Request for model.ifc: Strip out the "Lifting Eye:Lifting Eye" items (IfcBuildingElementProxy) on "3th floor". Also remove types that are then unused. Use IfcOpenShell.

First a look at what the model holds.

```python
import ifcopenshell
import ifcopenshell.util.element

model = ifcopenshell.open("model.ifc")
print(model.schema)
storey = next(s for s in model.by_type("IfcBuildingStorey") if s.Name == "3th floor")
proxies = [e for e in ifcopenshell.util.element.get_decomposition(storey) if e.is_a("IfcBuildingElementProxy")]
seen = {}
for e in proxies:
    element_type = ifcopenshell.util.element.get_type(e)
    name = element_type.Name if element_type not in (None, e) else None
    seen[name] = seen.get(name, 0) + 1
for name, count in sorted(seen.items(), key=str):
    print(count, "x", name)
```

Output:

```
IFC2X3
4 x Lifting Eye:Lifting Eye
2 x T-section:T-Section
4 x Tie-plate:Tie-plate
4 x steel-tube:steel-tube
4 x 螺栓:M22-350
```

```python
import ifcopenshell
import ifcopenshell.api.root
import ifcopenshell.util.element

model = ifcopenshell.open("model.ifc")

storey = next(s for s in model.by_type("IfcBuildingStorey") if s.Name == "3th floor")
proxies = [e for e in ifcopenshell.util.element.get_decomposition(storey) if e.is_a("IfcBuildingElementProxy")]
targets = [e for e in proxies if (t := ifcopenshell.util.element.get_type(e)) not in (None, e) and t.Name == "Lifting Eye:Lifting Eye"]
types = {ifcopenshell.util.element.get_type(e) for e in targets} - {None, *targets}

for e in targets:
    ifcopenshell.api.root.remove_product(model, product=e)
print(len(targets), "removed")

unused = [t for t in types if not ifcopenshell.util.element.get_types(t)]
for t in unused:
    ifcopenshell.api.root.remove_product(model, product=t)
print(len(unused), "unused types removed")

model.write("model_updated.ifc")
```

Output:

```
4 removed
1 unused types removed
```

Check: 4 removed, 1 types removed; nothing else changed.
